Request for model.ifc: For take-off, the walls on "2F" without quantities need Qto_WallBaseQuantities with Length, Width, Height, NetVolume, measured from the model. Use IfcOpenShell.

First a look at what the model holds.

```python
import ifcopenshell
import ifcopenshell.util.element
import ifcopenshell.util.unit

model = ifcopenshell.open("model.ifc")
print(model.schema)
for unit_type in ("LENGTHUNIT", "AREAUNIT", "VOLUMEUNIT"):
    print(unit_type, ifcopenshell.util.unit.calculate_unit_scale(model, unit_type))
storey = next(s for s in model.by_type("IfcBuildingStorey") if s.Name == "2F")
walls = [e for e in ifcopenshell.util.element.get_decomposition(storey) if e.is_a("IfcWall")]
for e in sorted(walls, key=lambda e: e.id()):
    print(e.id(), e.is_a(), e.Name, list(ifcopenshell.util.element.get_psets(e, qtos_only=True)), sep=" | ")
```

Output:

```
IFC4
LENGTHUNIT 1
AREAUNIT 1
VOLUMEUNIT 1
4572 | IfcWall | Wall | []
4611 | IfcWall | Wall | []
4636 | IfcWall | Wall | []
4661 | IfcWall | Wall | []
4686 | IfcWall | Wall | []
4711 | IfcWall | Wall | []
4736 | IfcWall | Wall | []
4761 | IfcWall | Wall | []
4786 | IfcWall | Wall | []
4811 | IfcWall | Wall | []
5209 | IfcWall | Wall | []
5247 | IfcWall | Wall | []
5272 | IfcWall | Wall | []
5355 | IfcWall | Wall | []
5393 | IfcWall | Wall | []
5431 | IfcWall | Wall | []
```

```python
import ifcopenshell
import ifcopenshell.api.pset
import ifcopenshell.geom
import ifcopenshell.util.element
import ifcopenshell.util.shape
import ifcopenshell.util.unit

model = ifcopenshell.open("model.ifc")
unit_scale = ifcopenshell.util.unit.calculate_unit_scale(model)
volume_scale = ifcopenshell.util.unit.calculate_unit_scale(model, "VOLUMEUNIT")
settings = ifcopenshell.geom.settings()

storey = next(s for s in model.by_type("IfcBuildingStorey") if s.Name == "2F")
walls = [e for e in ifcopenshell.util.element.get_decomposition(storey) if e.is_a("IfcWall")]

for e in sorted(walls, key=lambda e: e.id()):
    if ifcopenshell.util.element.get_psets(e, qtos_only=True, should_inherit=False):
        continue
    # Geometry comes back in metres, in the element's own axes.
    shape = ifcopenshell.geom.create_shape(settings, e)
    values = {
        "Length": ifcopenshell.util.shape.get_x(shape.geometry) / unit_scale,
        "Width": ifcopenshell.util.shape.get_y(shape.geometry) / unit_scale,
        "Height": ifcopenshell.util.shape.get_z(shape.geometry) / unit_scale,
        "NetVolume": ifcopenshell.util.shape.get_volume(shape.geometry) / volume_scale,
    }
    qto = ifcopenshell.api.pset.add_qto(model, product=e, name="Qto_WallBaseQuantities")
    ifcopenshell.api.pset.edit_qto(model, qto=qto, properties=values)
    print(e.id(), {k: round(v, 3) for k, v in values.items()})

model.write("model_edited.ifc")
```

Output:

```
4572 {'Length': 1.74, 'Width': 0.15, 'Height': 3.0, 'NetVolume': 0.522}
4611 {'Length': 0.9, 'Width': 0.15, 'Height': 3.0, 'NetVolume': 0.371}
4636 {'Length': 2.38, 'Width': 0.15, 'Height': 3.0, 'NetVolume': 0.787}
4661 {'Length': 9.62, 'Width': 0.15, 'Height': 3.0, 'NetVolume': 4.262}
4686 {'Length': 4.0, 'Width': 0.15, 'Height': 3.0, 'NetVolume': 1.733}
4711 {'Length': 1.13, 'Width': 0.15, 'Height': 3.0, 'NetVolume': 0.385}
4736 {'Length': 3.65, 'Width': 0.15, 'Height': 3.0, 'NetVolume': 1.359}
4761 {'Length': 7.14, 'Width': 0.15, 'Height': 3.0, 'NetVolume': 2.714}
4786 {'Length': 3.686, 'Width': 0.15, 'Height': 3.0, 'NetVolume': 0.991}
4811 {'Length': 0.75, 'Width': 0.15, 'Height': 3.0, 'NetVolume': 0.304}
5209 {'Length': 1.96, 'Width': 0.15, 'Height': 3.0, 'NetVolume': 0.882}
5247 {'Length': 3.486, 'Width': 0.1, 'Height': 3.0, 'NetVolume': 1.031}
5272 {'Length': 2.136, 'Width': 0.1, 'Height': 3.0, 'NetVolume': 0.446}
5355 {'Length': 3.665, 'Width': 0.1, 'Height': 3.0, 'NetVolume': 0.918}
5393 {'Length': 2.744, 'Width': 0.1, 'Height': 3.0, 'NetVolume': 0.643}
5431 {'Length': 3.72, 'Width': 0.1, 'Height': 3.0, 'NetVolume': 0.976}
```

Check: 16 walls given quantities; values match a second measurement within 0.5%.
